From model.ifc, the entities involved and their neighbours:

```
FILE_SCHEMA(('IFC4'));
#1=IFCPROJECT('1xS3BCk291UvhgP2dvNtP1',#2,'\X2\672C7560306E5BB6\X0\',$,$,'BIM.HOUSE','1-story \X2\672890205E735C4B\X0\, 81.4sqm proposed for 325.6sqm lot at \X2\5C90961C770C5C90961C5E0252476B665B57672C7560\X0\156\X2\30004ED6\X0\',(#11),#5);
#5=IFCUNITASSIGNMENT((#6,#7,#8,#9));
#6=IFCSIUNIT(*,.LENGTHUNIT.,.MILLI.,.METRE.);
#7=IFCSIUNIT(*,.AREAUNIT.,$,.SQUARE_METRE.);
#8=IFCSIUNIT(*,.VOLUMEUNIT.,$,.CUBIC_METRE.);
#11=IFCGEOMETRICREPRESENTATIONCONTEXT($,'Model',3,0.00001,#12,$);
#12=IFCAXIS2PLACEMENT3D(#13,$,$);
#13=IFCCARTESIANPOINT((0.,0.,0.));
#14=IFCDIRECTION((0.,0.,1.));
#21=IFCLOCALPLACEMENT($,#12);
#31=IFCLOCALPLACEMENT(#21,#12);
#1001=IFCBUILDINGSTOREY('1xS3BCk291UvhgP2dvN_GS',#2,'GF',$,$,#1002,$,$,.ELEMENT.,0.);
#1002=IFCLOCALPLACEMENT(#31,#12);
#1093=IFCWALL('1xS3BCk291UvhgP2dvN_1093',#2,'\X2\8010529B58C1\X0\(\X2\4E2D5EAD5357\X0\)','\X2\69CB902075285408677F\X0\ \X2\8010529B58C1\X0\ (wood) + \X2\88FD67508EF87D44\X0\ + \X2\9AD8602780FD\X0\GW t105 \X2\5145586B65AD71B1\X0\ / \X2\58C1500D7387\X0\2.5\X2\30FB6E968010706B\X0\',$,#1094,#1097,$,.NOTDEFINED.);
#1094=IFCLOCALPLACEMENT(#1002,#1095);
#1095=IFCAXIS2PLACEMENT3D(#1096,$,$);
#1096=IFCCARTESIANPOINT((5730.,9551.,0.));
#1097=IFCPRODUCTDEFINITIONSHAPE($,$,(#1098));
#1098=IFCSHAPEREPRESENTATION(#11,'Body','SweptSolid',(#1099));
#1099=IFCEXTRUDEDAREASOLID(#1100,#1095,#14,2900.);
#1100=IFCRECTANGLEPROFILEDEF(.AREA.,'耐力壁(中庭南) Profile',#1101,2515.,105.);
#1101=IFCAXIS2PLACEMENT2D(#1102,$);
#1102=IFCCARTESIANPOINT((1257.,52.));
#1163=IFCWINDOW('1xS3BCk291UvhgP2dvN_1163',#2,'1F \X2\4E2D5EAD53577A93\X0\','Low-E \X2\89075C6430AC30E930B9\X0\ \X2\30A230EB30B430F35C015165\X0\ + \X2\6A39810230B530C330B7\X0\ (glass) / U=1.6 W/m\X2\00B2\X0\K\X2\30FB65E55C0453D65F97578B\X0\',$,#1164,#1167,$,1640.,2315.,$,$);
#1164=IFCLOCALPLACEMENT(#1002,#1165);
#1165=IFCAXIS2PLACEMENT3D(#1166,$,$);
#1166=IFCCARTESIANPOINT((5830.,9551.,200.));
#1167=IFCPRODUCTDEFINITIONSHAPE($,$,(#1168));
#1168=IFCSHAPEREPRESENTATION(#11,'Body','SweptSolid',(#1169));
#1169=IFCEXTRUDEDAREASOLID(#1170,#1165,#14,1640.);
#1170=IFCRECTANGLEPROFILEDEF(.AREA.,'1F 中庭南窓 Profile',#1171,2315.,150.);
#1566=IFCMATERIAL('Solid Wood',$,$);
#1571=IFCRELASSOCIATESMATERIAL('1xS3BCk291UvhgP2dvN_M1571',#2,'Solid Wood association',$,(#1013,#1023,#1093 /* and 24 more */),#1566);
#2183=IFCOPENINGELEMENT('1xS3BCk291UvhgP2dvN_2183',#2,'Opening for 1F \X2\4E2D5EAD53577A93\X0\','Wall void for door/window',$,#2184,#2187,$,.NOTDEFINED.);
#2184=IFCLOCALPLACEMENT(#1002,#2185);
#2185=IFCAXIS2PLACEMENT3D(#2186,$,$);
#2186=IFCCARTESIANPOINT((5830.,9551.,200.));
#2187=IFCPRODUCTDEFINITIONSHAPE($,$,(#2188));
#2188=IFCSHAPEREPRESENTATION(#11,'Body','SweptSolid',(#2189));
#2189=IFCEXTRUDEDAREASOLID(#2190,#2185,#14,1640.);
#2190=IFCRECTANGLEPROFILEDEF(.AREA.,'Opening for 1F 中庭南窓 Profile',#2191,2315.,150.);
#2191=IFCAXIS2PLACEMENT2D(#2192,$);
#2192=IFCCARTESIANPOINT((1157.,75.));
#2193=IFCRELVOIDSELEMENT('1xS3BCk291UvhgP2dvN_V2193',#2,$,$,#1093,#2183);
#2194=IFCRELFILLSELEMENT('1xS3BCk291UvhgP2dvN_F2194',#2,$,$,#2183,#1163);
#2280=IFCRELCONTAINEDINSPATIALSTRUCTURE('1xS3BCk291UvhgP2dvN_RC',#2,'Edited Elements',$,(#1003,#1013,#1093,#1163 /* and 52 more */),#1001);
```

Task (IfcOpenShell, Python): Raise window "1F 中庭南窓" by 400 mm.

```python
import numpy as np
import ifcopenshell
import ifcopenshell.api.geometry
import ifcopenshell.util.placement
import ifcopenshell.util.unit

model = ifcopenshell.open("model.ifc")
unit_scale = ifcopenshell.util.unit.calculate_unit_scale(model)

window = model.by_id(1163)
opening = window.FillsVoids[0].RelatingOpeningElement
dz = 0.4 / unit_scale

shift = np.array([0.0, 0.0, dz])
# The window is not placed relative to its opening, so move both.
for product in (opening, window):
    matrix = ifcopenshell.util.placement.get_local_placement(product.ObjectPlacement)
    matrix[:3, 3] += shift
    ifcopenshell.api.geometry.edit_object_placement(model, product=product, matrix=matrix, is_si=False)

print(f"moved by {dz * unit_scale:+.3f} m")

model.write("model_rev.ifc")
```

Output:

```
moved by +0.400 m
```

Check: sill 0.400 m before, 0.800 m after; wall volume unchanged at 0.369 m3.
